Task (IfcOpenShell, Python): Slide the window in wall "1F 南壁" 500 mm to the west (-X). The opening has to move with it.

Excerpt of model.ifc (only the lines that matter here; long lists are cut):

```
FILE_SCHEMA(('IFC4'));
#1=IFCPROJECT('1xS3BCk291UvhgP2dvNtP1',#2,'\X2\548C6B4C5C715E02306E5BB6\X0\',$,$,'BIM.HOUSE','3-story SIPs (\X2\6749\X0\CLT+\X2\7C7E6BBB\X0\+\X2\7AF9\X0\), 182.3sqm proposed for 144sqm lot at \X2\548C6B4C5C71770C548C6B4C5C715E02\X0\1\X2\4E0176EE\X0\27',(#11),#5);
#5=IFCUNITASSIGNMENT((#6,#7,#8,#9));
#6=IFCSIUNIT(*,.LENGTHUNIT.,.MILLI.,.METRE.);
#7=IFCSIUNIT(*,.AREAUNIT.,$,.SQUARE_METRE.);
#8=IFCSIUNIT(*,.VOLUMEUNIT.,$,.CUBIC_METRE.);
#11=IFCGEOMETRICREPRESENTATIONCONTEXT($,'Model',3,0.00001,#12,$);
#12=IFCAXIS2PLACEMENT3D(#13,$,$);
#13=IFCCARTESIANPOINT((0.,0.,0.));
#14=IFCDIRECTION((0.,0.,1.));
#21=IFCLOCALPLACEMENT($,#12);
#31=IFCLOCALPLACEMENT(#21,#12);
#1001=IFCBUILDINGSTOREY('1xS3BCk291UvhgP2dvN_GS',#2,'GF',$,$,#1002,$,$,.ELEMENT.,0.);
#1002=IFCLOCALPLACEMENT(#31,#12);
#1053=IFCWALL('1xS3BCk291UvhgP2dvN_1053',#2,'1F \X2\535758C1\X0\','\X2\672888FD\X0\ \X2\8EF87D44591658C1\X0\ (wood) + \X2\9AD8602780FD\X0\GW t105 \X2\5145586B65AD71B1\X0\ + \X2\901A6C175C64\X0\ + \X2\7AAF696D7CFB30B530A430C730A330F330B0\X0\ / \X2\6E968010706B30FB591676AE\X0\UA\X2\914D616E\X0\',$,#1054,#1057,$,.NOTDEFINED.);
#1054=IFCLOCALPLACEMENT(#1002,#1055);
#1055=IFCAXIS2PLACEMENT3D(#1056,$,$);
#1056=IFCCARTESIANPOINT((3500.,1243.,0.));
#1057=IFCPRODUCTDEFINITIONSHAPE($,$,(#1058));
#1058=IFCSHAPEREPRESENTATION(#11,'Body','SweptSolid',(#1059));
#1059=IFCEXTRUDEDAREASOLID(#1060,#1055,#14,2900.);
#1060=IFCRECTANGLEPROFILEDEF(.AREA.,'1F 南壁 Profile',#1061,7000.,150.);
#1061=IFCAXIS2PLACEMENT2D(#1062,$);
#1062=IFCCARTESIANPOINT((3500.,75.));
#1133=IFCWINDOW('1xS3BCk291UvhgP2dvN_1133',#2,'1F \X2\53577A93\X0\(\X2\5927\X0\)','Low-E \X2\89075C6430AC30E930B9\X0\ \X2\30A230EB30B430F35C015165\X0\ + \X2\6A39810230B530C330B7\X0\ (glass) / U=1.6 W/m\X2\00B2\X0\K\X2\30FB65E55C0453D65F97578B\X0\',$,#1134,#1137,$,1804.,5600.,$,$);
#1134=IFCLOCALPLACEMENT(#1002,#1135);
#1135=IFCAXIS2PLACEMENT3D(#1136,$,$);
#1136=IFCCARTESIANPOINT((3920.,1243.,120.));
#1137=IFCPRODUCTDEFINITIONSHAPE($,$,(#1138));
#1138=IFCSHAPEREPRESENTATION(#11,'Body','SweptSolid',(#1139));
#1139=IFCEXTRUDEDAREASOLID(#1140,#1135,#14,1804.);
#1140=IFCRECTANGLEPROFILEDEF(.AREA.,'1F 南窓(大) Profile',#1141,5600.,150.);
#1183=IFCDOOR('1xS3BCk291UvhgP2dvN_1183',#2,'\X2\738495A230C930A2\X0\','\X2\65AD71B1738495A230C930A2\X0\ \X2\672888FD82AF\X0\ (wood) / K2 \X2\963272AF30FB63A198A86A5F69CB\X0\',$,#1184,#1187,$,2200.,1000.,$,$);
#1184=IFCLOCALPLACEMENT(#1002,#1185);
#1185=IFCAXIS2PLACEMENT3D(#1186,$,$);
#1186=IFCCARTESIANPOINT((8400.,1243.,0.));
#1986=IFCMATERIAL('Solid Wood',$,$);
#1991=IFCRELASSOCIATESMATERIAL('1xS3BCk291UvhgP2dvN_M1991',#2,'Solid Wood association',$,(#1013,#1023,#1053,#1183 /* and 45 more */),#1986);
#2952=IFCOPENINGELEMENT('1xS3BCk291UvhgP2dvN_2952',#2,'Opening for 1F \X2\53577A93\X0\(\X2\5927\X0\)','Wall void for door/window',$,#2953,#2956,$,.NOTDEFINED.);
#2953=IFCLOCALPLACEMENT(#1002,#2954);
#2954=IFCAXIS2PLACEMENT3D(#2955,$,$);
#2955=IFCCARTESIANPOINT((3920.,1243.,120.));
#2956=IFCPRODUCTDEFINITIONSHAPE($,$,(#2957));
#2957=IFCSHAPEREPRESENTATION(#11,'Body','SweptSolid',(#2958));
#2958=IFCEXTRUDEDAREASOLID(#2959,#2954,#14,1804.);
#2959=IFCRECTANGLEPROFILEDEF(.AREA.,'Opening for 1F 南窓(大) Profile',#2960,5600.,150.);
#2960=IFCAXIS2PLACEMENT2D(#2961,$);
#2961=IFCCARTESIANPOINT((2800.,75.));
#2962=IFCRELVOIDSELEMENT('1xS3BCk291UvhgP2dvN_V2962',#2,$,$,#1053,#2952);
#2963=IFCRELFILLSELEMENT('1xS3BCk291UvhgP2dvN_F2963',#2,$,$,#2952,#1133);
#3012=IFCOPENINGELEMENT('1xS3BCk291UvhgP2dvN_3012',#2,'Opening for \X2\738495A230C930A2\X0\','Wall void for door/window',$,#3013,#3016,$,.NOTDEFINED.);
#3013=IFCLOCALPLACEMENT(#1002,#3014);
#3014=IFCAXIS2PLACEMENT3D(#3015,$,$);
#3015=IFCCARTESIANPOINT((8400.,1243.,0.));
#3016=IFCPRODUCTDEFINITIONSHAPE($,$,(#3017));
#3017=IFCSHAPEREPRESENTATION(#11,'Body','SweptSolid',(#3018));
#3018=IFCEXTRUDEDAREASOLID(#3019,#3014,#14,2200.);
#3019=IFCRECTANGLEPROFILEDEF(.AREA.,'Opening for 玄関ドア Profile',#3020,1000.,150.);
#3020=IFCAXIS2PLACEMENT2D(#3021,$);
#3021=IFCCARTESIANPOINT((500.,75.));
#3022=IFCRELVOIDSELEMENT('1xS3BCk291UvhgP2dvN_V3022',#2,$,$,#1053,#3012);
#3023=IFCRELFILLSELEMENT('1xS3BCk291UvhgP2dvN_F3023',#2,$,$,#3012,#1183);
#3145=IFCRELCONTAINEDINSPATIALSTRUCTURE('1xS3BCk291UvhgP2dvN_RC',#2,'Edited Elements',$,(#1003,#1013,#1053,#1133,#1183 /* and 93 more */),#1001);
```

```python
import ifcopenshell
import ifcopenshell.api.geometry
import ifcopenshell.util.placement

model = ifcopenshell.open("model.ifc")

window = model.by_id(1133)
opening = window.FillsVoids[0].RelatingOpeningElement
wall = opening.VoidsElements[0].RelatingBuildingElement

wall_matrix = ifcopenshell.util.placement.get_local_placement(wall.ObjectPlacement)
shift = wall_matrix[:3, 0] * -500.0
before = ifcopenshell.util.placement.get_local_placement(window.ObjectPlacement)[:3, 3].copy()

# The window is not placed relative to its opening, so move both.
for product in (opening, window):
    matrix = ifcopenshell.util.placement.get_local_placement(product.ObjectPlacement)
    matrix[:3, 3] += shift
    ifcopenshell.api.geometry.edit_object_placement(model, product=product, matrix=matrix, is_si=False)

after = ifcopenshell.util.placement.get_local_placement(window.ObjectPlacement)[:3, 3]
print("window moved by", (after - before).round(3) + 0.0)

model.write("model_v2.ifc")
```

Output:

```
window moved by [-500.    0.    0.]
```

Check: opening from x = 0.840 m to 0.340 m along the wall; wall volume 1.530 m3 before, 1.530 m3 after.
